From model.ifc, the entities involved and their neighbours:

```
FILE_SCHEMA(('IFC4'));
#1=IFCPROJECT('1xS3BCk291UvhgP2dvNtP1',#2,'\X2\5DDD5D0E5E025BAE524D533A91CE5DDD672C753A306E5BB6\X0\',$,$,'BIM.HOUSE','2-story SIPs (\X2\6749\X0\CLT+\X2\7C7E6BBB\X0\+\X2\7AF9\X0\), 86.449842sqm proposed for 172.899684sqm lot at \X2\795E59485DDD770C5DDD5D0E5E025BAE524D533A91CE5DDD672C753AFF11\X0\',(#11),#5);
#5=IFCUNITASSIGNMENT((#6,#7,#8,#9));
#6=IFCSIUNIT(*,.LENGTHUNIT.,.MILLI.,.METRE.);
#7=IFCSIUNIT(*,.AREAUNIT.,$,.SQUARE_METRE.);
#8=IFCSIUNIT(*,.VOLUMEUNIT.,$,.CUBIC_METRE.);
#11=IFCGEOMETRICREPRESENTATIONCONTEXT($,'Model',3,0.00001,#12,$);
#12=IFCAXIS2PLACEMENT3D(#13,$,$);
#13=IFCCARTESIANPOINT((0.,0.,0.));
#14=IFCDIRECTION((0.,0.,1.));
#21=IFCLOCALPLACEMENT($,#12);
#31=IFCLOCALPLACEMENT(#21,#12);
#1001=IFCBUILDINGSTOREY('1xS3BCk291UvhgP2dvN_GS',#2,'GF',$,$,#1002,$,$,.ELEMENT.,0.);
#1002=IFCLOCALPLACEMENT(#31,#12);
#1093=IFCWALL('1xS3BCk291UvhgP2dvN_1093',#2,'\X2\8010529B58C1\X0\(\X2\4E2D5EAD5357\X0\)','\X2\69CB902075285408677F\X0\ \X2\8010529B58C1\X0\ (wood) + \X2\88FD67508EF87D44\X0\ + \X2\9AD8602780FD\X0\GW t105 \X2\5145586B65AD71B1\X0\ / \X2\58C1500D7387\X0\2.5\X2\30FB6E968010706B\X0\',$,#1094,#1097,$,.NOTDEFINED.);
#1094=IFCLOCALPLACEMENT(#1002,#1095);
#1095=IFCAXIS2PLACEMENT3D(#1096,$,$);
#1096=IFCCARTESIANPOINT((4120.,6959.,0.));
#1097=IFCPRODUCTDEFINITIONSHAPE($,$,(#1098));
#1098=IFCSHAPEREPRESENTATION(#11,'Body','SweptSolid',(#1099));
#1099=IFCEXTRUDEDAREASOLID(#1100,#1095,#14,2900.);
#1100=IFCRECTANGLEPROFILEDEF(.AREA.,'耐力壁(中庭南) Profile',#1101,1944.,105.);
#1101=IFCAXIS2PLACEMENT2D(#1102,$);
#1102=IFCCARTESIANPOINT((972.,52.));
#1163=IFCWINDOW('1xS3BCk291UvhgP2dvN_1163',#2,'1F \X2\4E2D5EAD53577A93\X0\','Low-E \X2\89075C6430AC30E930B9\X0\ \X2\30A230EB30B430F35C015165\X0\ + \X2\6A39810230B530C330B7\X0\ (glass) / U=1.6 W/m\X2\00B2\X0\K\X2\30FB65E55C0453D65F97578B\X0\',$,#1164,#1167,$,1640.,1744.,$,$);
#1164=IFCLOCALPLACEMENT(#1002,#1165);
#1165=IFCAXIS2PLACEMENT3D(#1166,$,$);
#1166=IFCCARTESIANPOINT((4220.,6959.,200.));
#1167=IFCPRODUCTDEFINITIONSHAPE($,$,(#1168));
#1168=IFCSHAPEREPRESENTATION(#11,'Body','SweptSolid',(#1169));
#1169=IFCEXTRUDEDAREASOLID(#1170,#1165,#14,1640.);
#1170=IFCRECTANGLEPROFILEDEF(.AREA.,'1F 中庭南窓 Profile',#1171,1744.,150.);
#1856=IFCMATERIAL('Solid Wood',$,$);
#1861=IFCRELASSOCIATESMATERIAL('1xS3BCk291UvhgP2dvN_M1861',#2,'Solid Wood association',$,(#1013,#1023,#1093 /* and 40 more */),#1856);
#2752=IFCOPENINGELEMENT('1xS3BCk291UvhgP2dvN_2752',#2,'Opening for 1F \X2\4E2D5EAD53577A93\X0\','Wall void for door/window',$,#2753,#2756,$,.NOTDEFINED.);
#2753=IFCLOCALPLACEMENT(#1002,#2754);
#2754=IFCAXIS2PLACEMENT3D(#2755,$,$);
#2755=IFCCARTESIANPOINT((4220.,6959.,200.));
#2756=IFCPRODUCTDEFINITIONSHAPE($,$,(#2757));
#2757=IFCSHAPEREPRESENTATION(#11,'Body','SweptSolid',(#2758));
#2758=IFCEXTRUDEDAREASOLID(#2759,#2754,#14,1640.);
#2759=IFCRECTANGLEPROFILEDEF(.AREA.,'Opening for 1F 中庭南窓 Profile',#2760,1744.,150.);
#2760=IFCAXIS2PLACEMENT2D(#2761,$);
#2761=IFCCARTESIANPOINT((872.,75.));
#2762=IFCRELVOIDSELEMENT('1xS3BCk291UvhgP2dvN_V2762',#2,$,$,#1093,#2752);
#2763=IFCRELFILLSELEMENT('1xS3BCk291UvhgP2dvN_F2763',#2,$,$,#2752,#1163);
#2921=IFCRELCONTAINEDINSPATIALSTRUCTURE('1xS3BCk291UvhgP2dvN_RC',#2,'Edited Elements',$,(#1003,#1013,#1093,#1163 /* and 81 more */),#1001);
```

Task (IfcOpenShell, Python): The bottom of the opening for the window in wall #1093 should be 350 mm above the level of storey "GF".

```python
import numpy as np
import ifcopenshell
import ifcopenshell.api.geometry
import ifcopenshell.geom
import ifcopenshell.util.element
import ifcopenshell.util.placement
import ifcopenshell.util.shape
import ifcopenshell.util.unit

model = ifcopenshell.open("model.ifc")
unit_scale = ifcopenshell.util.unit.calculate_unit_scale(model)

window = model.by_id(1163)
opening = window.FillsVoids[0].RelatingOpeningElement
storey = ifcopenshell.util.element.get_container(window, ifc_class="IfcBuildingStorey")
level = ifcopenshell.util.placement.get_local_placement(storey.ObjectPlacement)[2, 3]

# The opening's origin need not be at the sill, so measure its lowest point.
shape = ifcopenshell.geom.create_shape(ifcopenshell.geom.settings(), opening)
bottom = ifcopenshell.util.shape.get_shape_bottom_elevation(shape, shape.geometry) / unit_scale
dz = level + 350.0 - bottom

shift = np.array([0.0, 0.0, dz])
# The window is not placed relative to its opening, so move both.
for product in (opening, window):
    matrix = ifcopenshell.util.placement.get_local_placement(product.ObjectPlacement)
    matrix[:3, 3] += shift
    ifcopenshell.api.geometry.edit_object_placement(model, product=product, matrix=matrix, is_si=False)

print(f"moved by {dz * unit_scale:+.3f} m")

model.write("model_edited.ifc")
```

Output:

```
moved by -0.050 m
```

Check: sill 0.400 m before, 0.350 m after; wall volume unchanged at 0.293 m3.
